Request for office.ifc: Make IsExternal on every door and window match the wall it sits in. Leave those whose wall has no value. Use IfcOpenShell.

First a look at what the model holds.

```python
import ifcopenshell
import ifcopenshell.util.element

model = ifcopenshell.open("office.ifc")
print(model.schema)
seen = {}
for e in model.by_type("IfcDoor") + model.by_type("IfcWindow"):
    if not e.FillsVoids:
        continue
    host = e.FillsVoids[0].RelatingOpeningElement.VoidsElements[0].RelatingBuildingElement
    own = ifcopenshell.util.element.get_pset(e, f"Pset_{e.is_a()[3:].removesuffix('StandardCase')}Common", "IsExternal")
    wall = ifcopenshell.util.element.get_pset(host, "Pset_WallCommon", "IsExternal")
    seen[e.is_a(), own, wall] = seen.get((e.is_a(), own, wall), 0) + 1
for (cls, own, wall), count in sorted(seen.items(), key=str):
    print(count, cls, "IsExternal:", own, "| host wall:", wall)
```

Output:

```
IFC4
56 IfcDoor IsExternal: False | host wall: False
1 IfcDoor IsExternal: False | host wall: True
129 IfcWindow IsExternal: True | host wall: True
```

```python
import ifcopenshell
import ifcopenshell.api.pset
import ifcopenshell.util.element

model = ifcopenshell.open("office.ifc")

count = 0
for ifc_class, pset_name in (("IfcDoor", "Pset_DoorCommon"), ("IfcWindow", "Pset_WindowCommon")):
    for e in model.by_type(ifc_class):
        if not e.FillsVoids:
            continue
        host = e.FillsVoids[0].RelatingOpeningElement.VoidsElements[0].RelatingBuildingElement
        external = ifcopenshell.util.element.get_pset(host, "Pset_WallCommon", "IsExternal")
        if external is None or ifcopenshell.util.element.get_pset(e, pset_name, "IsExternal") == external:
            continue
        pset = ifcopenshell.api.pset.add_pset(model, product=e, name=pset_name)
        ifcopenshell.api.pset.edit_pset(model, pset=pset, properties={"IsExternal": external})
        count += 1

print(count, "updated")

model.write("office_updated.ifc")
```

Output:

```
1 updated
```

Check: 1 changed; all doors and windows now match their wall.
